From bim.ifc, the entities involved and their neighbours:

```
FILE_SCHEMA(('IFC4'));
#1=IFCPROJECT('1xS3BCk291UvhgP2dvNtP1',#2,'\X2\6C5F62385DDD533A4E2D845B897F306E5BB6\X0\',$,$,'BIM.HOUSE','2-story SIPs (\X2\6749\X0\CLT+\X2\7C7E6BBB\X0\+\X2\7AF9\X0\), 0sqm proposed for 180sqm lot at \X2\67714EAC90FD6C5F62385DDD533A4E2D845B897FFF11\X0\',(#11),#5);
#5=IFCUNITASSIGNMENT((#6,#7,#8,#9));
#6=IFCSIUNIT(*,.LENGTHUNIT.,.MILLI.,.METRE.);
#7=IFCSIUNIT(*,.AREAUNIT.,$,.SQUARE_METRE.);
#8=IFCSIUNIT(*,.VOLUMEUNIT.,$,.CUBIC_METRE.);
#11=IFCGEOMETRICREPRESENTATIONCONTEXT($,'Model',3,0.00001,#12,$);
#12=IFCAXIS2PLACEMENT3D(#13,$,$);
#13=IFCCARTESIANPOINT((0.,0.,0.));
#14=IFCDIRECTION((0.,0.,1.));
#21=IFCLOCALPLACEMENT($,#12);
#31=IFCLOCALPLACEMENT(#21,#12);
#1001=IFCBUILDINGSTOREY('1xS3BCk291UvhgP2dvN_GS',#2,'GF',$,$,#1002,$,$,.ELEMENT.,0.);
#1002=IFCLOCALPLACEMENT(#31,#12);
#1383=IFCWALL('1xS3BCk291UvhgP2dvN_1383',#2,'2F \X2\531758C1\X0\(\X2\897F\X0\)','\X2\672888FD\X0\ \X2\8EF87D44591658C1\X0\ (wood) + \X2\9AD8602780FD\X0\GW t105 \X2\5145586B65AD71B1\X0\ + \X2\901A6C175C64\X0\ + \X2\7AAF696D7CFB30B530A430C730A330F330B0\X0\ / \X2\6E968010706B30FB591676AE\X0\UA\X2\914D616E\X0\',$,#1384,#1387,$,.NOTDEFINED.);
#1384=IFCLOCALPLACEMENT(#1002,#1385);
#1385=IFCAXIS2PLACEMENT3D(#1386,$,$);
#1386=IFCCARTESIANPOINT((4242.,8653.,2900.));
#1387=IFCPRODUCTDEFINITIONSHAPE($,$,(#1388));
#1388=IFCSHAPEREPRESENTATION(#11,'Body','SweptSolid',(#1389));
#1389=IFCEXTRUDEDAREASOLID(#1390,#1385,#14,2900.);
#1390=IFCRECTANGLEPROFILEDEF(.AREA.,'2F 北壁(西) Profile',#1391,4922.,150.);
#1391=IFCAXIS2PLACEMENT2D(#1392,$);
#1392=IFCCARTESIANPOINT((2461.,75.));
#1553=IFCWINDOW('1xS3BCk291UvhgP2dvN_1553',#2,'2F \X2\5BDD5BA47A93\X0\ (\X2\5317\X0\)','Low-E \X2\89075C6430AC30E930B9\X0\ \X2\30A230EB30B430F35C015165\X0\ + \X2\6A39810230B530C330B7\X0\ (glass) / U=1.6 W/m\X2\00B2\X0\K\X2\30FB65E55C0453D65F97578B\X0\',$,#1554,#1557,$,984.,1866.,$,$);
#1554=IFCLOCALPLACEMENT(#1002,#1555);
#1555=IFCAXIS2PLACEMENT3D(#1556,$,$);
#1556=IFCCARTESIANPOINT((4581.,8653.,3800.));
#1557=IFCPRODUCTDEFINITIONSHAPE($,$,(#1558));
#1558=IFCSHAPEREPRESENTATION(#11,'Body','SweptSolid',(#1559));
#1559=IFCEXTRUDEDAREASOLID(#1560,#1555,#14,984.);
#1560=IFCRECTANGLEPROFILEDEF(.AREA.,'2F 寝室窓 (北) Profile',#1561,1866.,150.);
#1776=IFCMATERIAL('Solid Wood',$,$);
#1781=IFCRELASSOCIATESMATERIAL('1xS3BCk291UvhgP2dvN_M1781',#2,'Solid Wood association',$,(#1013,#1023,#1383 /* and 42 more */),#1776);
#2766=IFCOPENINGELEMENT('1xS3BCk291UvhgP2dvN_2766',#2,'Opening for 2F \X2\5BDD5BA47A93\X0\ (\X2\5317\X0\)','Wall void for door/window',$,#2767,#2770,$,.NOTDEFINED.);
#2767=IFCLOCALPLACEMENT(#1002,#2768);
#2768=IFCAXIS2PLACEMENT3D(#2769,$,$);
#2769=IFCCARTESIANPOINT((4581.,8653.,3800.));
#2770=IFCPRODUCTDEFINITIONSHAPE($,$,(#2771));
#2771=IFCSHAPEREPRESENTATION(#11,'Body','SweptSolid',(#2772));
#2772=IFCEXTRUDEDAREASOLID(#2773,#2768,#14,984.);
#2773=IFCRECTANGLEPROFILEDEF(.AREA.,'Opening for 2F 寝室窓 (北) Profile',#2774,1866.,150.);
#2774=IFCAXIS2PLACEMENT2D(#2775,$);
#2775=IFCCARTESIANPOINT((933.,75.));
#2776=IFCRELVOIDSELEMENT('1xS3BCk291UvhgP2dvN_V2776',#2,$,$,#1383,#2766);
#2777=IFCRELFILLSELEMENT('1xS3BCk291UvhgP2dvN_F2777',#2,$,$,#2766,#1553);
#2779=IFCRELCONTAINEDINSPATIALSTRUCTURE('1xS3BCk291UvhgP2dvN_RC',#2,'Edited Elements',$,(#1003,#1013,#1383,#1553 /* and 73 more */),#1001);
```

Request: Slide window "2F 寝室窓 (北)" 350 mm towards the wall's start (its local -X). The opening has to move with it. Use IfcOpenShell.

```python
import ifcopenshell
import ifcopenshell.api.geometry
import ifcopenshell.util.placement
import ifcopenshell.util.unit

model = ifcopenshell.open("bim.ifc")
unit_scale = ifcopenshell.util.unit.calculate_unit_scale(model)

window = model.by_guid("1xS3BCk291UvhgP2dvN_1553")
opening = window.FillsVoids[0].RelatingOpeningElement
wall = opening.VoidsElements[0].RelatingBuildingElement

wall_matrix = ifcopenshell.util.placement.get_local_placement(wall.ObjectPlacement)
shift = wall_matrix[:3, 0] * -0.35 / unit_scale
before = ifcopenshell.util.placement.get_local_placement(window.ObjectPlacement)[:3, 3].copy()

# The window is not placed relative to its opening, so move both.
for product in (opening, window):
    matrix = ifcopenshell.util.placement.get_local_placement(product.ObjectPlacement)
    matrix[:3, 3] += shift
    ifcopenshell.api.geometry.edit_object_placement(model, product=product, matrix=matrix, is_si=False)

after = ifcopenshell.util.placement.get_local_placement(window.ObjectPlacement)[:3, 3]
print("window moved by", (after - before).round(3) + 0.0)

model.write("bim_updated.ifc")
```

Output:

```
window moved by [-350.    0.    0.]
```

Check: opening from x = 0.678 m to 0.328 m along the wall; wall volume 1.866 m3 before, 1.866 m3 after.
